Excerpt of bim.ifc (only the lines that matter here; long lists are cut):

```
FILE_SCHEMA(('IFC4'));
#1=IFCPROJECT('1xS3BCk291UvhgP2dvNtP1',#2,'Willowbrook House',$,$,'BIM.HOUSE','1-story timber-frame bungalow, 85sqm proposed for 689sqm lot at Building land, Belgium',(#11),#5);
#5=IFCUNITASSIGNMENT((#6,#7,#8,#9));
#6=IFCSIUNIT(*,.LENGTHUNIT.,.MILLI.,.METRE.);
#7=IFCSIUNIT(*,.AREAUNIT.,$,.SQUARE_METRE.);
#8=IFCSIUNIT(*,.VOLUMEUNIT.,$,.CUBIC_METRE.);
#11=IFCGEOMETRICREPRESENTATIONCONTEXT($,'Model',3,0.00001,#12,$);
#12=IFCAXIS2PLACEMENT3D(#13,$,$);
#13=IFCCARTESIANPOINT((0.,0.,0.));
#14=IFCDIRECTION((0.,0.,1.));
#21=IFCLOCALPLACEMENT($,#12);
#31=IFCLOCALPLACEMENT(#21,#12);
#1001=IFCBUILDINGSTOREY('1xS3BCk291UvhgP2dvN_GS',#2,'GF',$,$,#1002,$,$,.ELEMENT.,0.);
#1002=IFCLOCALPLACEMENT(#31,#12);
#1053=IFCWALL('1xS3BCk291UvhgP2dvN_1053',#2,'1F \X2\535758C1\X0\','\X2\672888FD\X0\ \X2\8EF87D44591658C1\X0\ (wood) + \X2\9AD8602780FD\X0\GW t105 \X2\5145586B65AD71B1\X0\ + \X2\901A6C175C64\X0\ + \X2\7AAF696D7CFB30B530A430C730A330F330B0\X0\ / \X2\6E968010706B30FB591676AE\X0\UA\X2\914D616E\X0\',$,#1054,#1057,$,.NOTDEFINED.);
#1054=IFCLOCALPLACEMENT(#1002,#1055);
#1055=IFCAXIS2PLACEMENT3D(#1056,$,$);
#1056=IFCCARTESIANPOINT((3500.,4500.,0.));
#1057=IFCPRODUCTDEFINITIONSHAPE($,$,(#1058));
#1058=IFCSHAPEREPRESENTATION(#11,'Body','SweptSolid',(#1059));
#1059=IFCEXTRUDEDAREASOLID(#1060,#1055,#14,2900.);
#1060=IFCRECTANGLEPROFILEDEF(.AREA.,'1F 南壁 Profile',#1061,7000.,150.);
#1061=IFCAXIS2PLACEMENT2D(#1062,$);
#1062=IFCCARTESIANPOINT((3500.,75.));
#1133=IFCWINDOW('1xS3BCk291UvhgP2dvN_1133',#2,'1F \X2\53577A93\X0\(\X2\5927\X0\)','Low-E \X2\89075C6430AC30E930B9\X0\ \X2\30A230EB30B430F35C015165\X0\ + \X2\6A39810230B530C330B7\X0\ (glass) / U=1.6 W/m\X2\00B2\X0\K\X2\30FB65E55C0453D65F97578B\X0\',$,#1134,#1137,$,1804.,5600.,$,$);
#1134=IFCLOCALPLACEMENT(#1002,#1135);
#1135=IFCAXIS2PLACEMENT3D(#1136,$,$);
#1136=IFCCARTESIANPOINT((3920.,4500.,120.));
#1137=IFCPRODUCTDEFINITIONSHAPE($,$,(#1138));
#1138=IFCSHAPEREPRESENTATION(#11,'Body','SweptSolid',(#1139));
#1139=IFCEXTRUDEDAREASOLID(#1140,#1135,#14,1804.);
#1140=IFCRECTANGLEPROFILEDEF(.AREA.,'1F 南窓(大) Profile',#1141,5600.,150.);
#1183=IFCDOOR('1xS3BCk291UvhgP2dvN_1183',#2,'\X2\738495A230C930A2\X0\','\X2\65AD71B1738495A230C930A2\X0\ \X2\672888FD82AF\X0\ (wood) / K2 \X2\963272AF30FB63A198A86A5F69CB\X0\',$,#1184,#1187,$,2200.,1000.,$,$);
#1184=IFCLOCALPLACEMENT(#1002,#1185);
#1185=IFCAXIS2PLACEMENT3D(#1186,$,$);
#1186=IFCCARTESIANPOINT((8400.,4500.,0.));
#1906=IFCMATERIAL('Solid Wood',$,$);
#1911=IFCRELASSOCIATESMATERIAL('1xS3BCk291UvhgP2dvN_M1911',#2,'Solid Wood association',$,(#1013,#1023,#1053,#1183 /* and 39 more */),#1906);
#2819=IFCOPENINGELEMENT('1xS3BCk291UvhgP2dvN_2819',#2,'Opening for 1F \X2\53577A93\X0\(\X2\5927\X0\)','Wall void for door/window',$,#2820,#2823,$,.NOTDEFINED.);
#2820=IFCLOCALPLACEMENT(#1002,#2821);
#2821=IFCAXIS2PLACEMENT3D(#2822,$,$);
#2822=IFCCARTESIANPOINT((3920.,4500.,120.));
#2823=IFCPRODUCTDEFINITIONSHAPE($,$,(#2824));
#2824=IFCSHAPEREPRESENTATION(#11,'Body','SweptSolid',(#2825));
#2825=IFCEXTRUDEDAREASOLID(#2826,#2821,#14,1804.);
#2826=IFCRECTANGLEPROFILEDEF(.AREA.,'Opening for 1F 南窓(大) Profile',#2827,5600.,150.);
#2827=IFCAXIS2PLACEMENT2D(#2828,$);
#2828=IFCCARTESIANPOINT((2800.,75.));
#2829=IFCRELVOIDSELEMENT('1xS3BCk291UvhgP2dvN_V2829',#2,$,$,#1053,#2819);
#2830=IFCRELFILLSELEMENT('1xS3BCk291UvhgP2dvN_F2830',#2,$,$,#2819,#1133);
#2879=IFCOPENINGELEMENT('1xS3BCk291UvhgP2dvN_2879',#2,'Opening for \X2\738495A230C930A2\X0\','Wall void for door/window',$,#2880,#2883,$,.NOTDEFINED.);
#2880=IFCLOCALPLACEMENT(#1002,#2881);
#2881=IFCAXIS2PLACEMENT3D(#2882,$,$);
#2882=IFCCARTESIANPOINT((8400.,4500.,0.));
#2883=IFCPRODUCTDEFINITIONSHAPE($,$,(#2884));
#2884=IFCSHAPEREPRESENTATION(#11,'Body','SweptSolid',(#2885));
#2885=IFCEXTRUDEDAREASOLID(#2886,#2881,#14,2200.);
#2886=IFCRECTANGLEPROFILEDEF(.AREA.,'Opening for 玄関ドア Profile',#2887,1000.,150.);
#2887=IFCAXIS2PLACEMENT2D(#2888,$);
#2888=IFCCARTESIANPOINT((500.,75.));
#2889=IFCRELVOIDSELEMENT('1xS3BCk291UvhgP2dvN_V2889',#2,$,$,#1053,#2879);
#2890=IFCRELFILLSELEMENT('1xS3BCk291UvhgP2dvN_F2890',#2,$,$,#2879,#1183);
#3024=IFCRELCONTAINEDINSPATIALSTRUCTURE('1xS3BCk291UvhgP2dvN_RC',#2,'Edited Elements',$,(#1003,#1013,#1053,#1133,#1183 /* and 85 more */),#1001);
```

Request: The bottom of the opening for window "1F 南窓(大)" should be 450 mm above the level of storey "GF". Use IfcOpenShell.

```python
import numpy as np
import ifcopenshell
import ifcopenshell.api.geometry
import ifcopenshell.geom
import ifcopenshell.util.element
import ifcopenshell.util.placement
import ifcopenshell.util.shape
import ifcopenshell.util.unit

model = ifcopenshell.open("bim.ifc")
unit_scale = ifcopenshell.util.unit.calculate_unit_scale(model)

window = model.by_guid("1xS3BCk291UvhgP2dvN_1133")
opening = window.FillsVoids[0].RelatingOpeningElement
storey = ifcopenshell.util.element.get_container(window, ifc_class="IfcBuildingStorey")
level = ifcopenshell.util.placement.get_local_placement(storey.ObjectPlacement)[2, 3]

# The opening's origin need not be at the sill, so measure its lowest point.
shape = ifcopenshell.geom.create_shape(ifcopenshell.geom.settings(), opening)
bottom = ifcopenshell.util.shape.get_shape_bottom_elevation(shape, shape.geometry) / unit_scale
dz = level + 450.0 - bottom

shift = np.array([0.0, 0.0, dz])
# The window is not placed relative to its opening, so move both.
for product in (opening, window):
    matrix = ifcopenshell.util.placement.get_local_placement(product.ObjectPlacement)
    matrix[:3, 3] += shift
    ifcopenshell.api.geometry.edit_object_placement(model, product=product, matrix=matrix, is_si=False)

print(f"moved by {dz * unit_scale:+.3f} m")

model.write("bim_v2.ifc")
```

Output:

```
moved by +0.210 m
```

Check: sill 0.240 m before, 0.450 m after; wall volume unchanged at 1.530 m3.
